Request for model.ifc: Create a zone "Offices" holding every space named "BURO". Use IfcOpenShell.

First a look at what the model holds.

```python
import ifcopenshell

model = ifcopenshell.open("model.ifc")
print(model.schema)
seen = {}
for space in model.by_type("IfcSpace"):
    seen[space.LongName] = seen.get(space.LongName, 0) + 1
for name, count in sorted(seen.items(), key=str):
    print(count, "x", name)
print("zones:", [z.Name for z in model.by_type("IfcZone")][:20])
```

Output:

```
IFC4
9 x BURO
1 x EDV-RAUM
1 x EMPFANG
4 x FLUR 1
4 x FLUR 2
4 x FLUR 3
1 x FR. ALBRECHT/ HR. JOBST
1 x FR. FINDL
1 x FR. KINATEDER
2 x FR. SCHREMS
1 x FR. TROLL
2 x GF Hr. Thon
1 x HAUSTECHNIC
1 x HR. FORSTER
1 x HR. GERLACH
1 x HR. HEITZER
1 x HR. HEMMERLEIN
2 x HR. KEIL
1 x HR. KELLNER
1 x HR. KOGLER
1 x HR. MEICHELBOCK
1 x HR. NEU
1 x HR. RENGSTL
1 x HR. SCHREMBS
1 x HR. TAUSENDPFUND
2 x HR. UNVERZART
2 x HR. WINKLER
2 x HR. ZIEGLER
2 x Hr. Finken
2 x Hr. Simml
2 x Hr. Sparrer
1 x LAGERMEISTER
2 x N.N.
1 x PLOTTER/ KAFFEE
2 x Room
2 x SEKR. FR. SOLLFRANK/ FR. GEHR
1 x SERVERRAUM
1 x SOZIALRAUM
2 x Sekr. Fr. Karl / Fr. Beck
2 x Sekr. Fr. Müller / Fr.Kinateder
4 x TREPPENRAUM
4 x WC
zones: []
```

```python
import ifcopenshell
import ifcopenshell.api.group
import ifcopenshell.api.root

model = ifcopenshell.open("model.ifc")

names = {"BURO"}
spaces = [s for s in model.by_type("IfcSpace") if s.LongName in names]

zone = ifcopenshell.api.root.create_entity(model, ifc_class="IfcZone", name="Offices")
ifcopenshell.api.group.assign_group(model, products=spaces, group=zone)
print(len(spaces), "spaces in", zone.Name)

model.write("model_rev.ifc")
```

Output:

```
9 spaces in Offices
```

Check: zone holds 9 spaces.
